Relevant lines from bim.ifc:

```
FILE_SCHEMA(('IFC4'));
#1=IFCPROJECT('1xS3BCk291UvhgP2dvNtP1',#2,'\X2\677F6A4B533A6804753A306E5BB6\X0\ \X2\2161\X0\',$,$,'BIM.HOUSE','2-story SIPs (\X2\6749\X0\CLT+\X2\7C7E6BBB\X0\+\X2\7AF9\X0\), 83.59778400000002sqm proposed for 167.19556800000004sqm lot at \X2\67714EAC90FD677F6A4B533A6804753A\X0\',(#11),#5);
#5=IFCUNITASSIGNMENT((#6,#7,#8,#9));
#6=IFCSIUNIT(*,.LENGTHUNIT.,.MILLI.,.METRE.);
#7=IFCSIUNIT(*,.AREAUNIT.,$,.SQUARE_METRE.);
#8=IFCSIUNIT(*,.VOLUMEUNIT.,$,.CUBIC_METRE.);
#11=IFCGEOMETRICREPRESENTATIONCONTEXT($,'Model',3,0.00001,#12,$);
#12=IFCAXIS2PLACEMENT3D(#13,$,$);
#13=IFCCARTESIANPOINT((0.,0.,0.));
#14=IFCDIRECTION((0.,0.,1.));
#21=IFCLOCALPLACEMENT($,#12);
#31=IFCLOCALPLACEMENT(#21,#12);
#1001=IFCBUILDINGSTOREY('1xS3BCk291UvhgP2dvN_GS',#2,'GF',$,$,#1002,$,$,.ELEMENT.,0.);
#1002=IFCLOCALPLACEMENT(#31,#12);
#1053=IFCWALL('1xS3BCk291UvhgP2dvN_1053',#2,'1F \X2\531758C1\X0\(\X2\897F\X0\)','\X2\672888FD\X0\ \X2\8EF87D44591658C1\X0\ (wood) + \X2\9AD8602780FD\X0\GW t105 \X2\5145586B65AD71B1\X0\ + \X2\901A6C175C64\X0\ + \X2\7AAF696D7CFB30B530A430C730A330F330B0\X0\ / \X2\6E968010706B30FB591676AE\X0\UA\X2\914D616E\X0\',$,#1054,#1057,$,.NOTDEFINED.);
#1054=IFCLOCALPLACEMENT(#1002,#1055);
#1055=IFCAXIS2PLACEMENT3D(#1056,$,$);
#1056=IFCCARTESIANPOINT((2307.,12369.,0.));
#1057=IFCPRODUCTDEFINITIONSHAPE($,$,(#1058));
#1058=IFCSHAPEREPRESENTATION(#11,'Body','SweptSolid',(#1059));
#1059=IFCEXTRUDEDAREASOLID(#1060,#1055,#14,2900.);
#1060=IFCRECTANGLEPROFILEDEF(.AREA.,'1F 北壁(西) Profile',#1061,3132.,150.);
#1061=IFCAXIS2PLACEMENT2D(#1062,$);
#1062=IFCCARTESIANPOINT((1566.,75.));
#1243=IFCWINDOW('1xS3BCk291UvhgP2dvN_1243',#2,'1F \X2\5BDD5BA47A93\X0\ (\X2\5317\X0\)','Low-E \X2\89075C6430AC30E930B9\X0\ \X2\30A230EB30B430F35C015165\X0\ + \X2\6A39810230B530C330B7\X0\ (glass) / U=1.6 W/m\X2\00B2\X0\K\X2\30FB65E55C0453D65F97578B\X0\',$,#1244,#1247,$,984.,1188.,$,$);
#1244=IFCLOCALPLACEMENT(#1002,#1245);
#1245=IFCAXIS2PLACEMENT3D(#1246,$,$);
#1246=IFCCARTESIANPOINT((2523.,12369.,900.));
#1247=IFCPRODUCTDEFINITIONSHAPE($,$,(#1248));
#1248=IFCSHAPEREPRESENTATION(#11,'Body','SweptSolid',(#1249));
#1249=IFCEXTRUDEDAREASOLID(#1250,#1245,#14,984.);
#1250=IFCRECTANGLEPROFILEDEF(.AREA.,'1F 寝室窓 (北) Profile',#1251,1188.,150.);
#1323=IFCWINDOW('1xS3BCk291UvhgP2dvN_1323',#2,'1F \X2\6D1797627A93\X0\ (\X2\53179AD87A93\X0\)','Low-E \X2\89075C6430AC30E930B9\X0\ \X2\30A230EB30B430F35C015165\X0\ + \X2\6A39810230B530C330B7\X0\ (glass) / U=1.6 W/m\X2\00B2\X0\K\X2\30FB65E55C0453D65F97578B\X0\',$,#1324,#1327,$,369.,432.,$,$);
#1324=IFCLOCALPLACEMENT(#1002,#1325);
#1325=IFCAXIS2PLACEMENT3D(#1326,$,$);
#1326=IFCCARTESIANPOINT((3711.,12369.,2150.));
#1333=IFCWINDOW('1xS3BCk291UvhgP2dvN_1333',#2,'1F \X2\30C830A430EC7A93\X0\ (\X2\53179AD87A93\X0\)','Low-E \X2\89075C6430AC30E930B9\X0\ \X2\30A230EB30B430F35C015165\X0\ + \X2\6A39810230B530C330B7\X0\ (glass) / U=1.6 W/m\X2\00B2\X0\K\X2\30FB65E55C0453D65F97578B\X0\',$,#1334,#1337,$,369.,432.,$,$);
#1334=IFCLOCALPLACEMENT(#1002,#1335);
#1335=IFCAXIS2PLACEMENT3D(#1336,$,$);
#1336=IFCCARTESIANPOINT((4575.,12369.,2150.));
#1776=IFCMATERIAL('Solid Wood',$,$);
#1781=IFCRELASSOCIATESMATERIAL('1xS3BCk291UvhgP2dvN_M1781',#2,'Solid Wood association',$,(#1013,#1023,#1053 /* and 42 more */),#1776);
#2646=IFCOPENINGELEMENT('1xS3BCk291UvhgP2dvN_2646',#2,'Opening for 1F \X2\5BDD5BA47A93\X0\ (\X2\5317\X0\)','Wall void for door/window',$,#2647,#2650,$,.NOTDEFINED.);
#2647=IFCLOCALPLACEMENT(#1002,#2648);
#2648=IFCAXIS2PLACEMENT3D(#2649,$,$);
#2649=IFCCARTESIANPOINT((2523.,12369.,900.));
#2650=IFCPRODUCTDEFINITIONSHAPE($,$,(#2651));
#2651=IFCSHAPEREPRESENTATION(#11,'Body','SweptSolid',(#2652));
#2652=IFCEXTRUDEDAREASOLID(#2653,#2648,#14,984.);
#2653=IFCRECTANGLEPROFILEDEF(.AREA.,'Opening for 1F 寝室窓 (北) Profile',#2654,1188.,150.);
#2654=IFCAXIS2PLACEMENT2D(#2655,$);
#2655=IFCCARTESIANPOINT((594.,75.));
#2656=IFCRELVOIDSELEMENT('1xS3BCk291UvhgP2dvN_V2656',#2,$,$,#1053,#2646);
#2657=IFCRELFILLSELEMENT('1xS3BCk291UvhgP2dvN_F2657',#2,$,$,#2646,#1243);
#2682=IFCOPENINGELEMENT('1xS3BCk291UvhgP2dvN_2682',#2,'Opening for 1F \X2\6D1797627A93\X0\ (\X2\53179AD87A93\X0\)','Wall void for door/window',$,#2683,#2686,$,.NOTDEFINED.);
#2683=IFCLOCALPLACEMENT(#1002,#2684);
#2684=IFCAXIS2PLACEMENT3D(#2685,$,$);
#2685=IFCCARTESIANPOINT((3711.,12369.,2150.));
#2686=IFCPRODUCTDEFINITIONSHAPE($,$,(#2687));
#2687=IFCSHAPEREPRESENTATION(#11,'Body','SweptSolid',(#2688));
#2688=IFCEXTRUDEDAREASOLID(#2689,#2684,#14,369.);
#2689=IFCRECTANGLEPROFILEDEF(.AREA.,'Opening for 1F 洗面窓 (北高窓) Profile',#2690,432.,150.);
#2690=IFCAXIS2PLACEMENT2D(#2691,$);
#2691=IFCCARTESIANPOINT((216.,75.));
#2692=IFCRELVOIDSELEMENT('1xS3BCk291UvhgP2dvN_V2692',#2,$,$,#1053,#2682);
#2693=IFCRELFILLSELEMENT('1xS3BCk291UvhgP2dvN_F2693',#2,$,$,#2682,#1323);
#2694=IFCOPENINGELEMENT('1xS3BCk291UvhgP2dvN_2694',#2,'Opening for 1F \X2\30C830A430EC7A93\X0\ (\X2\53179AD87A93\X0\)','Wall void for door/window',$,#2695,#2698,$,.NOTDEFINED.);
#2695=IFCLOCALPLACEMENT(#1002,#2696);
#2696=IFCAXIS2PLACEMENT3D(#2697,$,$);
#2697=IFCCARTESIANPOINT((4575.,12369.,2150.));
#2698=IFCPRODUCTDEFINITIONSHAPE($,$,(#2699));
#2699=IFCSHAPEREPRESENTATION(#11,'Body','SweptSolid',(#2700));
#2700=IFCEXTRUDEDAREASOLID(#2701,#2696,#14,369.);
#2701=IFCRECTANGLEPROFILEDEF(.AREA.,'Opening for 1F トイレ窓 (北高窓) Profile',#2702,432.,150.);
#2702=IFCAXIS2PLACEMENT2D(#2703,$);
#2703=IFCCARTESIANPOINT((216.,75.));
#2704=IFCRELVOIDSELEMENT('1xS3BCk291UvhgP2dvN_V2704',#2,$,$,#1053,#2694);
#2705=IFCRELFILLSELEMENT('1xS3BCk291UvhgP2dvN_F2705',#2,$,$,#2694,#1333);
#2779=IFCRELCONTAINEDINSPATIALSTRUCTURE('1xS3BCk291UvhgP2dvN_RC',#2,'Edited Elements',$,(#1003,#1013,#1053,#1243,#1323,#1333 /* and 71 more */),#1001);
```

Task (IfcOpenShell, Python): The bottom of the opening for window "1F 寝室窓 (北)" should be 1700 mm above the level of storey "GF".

```python
import numpy as np
import ifcopenshell
import ifcopenshell.api.geometry
import ifcopenshell.geom
import ifcopenshell.util.element
import ifcopenshell.util.placement
import ifcopenshell.util.shape
import ifcopenshell.util.unit

model = ifcopenshell.open("bim.ifc")
unit_scale = ifcopenshell.util.unit.calculate_unit_scale(model)

window = model.by_guid("1xS3BCk291UvhgP2dvN_1243")
opening = window.FillsVoids[0].RelatingOpeningElement
storey = ifcopenshell.util.element.get_container(window, ifc_class="IfcBuildingStorey")
level = ifcopenshell.util.placement.get_local_placement(storey.ObjectPlacement)[2, 3]

# The opening's origin need not be at the sill, so measure its lowest point.
shape = ifcopenshell.geom.create_shape(ifcopenshell.geom.settings(), opening)
bottom = ifcopenshell.util.shape.get_shape_bottom_elevation(shape, shape.geometry) / unit_scale
dz = level + 1.7 / unit_scale - bottom

shift = np.array([0.0, 0.0, dz])
# The window is not placed relative to its opening, so move both.
for product in (opening, window):
    matrix = ifcopenshell.util.placement.get_local_placement(product.ObjectPlacement)
    matrix[:3, 3] += shift
    ifcopenshell.api.geometry.edit_object_placement(model, product=product, matrix=matrix, is_si=False)

print(f"moved by {dz * unit_scale:+.3f} m")

model.write("bim_updated.ifc")
```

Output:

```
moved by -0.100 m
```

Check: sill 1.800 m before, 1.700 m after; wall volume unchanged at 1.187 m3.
